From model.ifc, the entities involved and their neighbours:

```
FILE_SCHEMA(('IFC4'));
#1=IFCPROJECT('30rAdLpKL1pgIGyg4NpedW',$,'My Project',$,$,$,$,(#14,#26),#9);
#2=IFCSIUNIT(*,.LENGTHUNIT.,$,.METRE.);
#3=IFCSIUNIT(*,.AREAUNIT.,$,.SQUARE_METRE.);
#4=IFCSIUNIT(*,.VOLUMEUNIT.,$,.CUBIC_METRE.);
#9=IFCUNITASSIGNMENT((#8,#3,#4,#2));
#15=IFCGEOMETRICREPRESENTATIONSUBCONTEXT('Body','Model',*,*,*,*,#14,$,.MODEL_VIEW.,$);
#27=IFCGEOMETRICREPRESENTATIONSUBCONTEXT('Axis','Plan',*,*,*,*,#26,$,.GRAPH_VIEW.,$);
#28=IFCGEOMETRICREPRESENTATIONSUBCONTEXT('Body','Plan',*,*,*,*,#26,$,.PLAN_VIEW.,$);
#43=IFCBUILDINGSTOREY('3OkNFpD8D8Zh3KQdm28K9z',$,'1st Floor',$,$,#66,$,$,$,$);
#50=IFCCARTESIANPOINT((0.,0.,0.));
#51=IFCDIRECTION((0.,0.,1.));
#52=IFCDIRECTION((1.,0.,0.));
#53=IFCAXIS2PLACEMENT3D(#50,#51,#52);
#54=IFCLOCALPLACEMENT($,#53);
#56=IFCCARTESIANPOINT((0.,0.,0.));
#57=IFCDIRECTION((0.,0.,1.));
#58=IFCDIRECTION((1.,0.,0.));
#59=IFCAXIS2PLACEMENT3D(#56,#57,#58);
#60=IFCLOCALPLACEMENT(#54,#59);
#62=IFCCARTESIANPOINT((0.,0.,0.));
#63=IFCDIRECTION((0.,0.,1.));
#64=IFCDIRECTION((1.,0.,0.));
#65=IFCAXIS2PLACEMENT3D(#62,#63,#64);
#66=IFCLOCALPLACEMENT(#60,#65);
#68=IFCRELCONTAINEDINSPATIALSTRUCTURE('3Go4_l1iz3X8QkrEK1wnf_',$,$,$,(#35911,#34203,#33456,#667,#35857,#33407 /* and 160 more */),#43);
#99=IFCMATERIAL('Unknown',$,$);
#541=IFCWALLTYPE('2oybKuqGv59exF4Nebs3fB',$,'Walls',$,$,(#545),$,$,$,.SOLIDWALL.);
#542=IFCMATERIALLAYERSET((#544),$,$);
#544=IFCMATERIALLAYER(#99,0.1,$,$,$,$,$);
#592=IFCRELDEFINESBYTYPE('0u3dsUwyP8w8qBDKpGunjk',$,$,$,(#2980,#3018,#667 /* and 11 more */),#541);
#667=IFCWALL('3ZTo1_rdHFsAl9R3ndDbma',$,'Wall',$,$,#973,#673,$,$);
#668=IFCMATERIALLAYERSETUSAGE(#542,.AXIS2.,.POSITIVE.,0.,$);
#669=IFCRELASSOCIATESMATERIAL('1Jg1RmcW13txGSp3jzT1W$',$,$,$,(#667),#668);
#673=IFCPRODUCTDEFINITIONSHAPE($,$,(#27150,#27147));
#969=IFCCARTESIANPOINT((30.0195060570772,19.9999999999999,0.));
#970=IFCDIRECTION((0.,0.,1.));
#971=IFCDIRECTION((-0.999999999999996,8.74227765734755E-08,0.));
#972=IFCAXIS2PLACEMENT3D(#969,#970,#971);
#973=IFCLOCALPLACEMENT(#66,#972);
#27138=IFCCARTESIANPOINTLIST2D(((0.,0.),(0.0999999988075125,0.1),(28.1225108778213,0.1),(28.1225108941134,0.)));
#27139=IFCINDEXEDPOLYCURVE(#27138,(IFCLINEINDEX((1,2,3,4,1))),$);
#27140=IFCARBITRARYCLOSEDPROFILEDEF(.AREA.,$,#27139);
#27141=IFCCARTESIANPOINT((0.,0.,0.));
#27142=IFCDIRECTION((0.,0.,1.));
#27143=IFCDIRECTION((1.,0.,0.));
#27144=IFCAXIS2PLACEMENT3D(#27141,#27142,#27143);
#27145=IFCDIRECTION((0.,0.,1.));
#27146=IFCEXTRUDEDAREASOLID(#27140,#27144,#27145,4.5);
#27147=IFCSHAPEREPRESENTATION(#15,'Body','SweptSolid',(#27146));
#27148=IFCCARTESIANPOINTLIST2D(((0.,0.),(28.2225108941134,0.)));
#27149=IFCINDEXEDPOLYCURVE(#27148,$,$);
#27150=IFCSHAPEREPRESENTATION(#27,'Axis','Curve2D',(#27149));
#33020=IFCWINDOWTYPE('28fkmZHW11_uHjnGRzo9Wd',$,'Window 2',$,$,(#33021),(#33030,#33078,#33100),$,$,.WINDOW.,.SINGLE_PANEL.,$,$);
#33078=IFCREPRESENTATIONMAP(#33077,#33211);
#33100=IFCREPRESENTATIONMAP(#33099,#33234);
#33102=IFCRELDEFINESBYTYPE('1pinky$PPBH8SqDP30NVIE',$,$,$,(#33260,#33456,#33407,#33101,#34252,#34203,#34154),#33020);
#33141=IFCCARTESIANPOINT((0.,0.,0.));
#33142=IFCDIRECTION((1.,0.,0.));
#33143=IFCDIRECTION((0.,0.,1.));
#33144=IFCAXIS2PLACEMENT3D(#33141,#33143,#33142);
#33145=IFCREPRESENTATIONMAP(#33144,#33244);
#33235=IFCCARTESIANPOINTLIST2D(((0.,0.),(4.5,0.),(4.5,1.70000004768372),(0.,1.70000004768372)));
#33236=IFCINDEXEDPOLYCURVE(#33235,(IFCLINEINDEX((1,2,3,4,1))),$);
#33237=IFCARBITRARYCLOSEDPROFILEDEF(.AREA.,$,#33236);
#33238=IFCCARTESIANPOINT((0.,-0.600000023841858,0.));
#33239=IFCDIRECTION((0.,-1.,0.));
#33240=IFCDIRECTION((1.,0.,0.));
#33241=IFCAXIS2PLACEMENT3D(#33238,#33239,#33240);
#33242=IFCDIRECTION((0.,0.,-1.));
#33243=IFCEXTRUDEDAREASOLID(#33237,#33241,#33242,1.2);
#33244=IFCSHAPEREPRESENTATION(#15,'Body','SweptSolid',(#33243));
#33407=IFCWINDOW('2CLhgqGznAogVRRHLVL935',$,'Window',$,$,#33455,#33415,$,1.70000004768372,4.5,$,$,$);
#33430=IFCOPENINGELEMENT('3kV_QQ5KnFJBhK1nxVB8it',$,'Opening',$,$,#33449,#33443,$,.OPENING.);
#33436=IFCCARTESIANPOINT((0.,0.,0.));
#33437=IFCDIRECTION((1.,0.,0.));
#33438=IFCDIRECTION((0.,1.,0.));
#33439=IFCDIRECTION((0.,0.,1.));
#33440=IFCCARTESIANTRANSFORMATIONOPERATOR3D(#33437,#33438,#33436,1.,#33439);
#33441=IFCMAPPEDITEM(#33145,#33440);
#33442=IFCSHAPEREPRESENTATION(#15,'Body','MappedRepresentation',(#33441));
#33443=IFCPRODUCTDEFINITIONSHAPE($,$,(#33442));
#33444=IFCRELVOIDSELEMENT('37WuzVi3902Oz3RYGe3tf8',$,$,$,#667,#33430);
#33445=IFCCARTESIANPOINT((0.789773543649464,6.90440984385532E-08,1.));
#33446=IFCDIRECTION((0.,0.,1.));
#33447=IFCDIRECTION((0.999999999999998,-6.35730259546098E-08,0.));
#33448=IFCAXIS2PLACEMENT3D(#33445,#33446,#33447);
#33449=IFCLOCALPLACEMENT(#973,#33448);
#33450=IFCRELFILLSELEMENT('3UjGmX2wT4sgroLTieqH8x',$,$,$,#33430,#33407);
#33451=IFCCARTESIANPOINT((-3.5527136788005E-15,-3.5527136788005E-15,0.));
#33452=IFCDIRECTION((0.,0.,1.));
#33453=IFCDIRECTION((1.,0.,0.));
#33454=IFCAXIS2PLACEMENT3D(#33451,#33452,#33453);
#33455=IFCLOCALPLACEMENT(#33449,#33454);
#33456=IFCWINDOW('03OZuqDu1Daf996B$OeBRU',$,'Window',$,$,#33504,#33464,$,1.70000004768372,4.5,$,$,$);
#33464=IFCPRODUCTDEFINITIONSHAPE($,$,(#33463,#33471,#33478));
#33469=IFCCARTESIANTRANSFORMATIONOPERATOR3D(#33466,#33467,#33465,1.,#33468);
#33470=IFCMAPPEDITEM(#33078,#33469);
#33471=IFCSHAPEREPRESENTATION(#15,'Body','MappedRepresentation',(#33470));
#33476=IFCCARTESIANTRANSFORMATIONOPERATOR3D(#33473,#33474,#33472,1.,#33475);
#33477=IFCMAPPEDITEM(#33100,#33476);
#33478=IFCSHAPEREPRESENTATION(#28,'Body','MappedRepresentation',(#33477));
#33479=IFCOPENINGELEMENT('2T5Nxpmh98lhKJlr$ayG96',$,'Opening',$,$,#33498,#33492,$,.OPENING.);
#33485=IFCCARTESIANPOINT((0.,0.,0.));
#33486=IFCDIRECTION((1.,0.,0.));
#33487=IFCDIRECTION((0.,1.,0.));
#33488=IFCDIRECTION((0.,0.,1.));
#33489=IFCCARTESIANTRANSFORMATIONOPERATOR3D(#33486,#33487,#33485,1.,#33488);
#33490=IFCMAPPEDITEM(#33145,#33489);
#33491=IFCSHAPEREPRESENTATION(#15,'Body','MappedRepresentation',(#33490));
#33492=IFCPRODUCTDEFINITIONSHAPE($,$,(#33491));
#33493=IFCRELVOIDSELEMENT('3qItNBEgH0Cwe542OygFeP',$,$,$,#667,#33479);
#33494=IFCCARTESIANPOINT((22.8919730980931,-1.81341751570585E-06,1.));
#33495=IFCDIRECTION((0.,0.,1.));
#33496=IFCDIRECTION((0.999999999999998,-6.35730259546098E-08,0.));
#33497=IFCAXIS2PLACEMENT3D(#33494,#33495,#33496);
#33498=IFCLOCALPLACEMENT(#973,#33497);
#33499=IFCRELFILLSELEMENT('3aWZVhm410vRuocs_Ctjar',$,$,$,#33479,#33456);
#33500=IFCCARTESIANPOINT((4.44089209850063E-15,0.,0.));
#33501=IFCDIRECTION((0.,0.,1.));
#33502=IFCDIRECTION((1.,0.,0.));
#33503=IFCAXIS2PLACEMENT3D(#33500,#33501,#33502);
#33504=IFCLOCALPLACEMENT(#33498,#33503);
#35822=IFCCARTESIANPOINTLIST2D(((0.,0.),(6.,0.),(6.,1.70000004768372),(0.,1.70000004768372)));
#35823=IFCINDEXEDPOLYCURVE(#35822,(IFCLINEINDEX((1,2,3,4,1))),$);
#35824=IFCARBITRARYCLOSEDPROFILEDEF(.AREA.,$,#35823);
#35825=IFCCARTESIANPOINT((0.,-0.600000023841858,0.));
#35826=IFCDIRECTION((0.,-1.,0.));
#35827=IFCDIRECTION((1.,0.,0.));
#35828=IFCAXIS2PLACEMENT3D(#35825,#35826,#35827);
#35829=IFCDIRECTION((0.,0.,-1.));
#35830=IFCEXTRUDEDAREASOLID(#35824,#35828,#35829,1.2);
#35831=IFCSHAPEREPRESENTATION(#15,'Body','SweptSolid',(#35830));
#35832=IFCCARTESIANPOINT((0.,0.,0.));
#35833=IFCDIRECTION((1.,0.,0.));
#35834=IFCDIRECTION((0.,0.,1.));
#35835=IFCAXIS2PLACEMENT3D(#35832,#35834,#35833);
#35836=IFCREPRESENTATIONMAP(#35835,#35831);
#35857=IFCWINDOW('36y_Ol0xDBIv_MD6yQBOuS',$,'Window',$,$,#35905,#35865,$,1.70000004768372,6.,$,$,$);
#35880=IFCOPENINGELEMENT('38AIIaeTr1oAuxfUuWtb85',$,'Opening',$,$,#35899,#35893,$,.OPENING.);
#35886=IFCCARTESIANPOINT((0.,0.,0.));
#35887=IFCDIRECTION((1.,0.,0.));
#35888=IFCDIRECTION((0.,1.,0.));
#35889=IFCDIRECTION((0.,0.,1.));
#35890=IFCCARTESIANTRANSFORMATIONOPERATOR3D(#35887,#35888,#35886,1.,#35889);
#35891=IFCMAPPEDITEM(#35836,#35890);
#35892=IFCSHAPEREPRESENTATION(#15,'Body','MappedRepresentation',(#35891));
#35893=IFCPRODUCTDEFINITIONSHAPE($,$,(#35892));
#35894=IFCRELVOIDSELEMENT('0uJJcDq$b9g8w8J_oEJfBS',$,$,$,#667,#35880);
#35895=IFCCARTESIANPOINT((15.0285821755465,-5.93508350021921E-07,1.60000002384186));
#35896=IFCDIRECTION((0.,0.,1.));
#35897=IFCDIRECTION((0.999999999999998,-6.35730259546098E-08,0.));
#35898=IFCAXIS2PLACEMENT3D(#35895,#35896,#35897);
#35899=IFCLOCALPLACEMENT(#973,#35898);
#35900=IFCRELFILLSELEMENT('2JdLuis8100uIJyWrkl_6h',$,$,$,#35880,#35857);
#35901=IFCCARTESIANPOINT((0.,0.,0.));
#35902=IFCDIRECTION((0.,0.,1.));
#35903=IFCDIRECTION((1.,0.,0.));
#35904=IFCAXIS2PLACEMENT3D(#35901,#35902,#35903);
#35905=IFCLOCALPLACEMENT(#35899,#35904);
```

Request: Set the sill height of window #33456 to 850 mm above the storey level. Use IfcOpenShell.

```python
import numpy as np
import ifcopenshell
import ifcopenshell.api.geometry
import ifcopenshell.geom
import ifcopenshell.util.element
import ifcopenshell.util.placement
import ifcopenshell.util.shape
import ifcopenshell.util.unit

model = ifcopenshell.open("model.ifc")
unit_scale = ifcopenshell.util.unit.calculate_unit_scale(model)

window = model.by_id(33456)
opening = window.FillsVoids[0].RelatingOpeningElement
storey = ifcopenshell.util.element.get_container(window, ifc_class="IfcBuildingStorey")
level = ifcopenshell.util.placement.get_local_placement(storey.ObjectPlacement)[2, 3]

# The opening's origin need not be at the sill, so measure its lowest point.
shape = ifcopenshell.geom.create_shape(ifcopenshell.geom.settings(), opening)
bottom = ifcopenshell.util.shape.get_shape_bottom_elevation(shape, shape.geometry) / unit_scale
dz = level + 0.85 - bottom

shift = np.array([0.0, 0.0, dz])
# The window is placed relative to its opening, so it follows when the opening moves.
matrix = ifcopenshell.util.placement.get_local_placement(opening.ObjectPlacement)
matrix[:3, 3] += shift
ifcopenshell.api.geometry.edit_object_placement(
    model, product=opening, matrix=matrix, is_si=False, should_transform_children=True
)

print(f"moved by {dz * unit_scale:+.3f} m")

model.write("model_rev.ifc")
```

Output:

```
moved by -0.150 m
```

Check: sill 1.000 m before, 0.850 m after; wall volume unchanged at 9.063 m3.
